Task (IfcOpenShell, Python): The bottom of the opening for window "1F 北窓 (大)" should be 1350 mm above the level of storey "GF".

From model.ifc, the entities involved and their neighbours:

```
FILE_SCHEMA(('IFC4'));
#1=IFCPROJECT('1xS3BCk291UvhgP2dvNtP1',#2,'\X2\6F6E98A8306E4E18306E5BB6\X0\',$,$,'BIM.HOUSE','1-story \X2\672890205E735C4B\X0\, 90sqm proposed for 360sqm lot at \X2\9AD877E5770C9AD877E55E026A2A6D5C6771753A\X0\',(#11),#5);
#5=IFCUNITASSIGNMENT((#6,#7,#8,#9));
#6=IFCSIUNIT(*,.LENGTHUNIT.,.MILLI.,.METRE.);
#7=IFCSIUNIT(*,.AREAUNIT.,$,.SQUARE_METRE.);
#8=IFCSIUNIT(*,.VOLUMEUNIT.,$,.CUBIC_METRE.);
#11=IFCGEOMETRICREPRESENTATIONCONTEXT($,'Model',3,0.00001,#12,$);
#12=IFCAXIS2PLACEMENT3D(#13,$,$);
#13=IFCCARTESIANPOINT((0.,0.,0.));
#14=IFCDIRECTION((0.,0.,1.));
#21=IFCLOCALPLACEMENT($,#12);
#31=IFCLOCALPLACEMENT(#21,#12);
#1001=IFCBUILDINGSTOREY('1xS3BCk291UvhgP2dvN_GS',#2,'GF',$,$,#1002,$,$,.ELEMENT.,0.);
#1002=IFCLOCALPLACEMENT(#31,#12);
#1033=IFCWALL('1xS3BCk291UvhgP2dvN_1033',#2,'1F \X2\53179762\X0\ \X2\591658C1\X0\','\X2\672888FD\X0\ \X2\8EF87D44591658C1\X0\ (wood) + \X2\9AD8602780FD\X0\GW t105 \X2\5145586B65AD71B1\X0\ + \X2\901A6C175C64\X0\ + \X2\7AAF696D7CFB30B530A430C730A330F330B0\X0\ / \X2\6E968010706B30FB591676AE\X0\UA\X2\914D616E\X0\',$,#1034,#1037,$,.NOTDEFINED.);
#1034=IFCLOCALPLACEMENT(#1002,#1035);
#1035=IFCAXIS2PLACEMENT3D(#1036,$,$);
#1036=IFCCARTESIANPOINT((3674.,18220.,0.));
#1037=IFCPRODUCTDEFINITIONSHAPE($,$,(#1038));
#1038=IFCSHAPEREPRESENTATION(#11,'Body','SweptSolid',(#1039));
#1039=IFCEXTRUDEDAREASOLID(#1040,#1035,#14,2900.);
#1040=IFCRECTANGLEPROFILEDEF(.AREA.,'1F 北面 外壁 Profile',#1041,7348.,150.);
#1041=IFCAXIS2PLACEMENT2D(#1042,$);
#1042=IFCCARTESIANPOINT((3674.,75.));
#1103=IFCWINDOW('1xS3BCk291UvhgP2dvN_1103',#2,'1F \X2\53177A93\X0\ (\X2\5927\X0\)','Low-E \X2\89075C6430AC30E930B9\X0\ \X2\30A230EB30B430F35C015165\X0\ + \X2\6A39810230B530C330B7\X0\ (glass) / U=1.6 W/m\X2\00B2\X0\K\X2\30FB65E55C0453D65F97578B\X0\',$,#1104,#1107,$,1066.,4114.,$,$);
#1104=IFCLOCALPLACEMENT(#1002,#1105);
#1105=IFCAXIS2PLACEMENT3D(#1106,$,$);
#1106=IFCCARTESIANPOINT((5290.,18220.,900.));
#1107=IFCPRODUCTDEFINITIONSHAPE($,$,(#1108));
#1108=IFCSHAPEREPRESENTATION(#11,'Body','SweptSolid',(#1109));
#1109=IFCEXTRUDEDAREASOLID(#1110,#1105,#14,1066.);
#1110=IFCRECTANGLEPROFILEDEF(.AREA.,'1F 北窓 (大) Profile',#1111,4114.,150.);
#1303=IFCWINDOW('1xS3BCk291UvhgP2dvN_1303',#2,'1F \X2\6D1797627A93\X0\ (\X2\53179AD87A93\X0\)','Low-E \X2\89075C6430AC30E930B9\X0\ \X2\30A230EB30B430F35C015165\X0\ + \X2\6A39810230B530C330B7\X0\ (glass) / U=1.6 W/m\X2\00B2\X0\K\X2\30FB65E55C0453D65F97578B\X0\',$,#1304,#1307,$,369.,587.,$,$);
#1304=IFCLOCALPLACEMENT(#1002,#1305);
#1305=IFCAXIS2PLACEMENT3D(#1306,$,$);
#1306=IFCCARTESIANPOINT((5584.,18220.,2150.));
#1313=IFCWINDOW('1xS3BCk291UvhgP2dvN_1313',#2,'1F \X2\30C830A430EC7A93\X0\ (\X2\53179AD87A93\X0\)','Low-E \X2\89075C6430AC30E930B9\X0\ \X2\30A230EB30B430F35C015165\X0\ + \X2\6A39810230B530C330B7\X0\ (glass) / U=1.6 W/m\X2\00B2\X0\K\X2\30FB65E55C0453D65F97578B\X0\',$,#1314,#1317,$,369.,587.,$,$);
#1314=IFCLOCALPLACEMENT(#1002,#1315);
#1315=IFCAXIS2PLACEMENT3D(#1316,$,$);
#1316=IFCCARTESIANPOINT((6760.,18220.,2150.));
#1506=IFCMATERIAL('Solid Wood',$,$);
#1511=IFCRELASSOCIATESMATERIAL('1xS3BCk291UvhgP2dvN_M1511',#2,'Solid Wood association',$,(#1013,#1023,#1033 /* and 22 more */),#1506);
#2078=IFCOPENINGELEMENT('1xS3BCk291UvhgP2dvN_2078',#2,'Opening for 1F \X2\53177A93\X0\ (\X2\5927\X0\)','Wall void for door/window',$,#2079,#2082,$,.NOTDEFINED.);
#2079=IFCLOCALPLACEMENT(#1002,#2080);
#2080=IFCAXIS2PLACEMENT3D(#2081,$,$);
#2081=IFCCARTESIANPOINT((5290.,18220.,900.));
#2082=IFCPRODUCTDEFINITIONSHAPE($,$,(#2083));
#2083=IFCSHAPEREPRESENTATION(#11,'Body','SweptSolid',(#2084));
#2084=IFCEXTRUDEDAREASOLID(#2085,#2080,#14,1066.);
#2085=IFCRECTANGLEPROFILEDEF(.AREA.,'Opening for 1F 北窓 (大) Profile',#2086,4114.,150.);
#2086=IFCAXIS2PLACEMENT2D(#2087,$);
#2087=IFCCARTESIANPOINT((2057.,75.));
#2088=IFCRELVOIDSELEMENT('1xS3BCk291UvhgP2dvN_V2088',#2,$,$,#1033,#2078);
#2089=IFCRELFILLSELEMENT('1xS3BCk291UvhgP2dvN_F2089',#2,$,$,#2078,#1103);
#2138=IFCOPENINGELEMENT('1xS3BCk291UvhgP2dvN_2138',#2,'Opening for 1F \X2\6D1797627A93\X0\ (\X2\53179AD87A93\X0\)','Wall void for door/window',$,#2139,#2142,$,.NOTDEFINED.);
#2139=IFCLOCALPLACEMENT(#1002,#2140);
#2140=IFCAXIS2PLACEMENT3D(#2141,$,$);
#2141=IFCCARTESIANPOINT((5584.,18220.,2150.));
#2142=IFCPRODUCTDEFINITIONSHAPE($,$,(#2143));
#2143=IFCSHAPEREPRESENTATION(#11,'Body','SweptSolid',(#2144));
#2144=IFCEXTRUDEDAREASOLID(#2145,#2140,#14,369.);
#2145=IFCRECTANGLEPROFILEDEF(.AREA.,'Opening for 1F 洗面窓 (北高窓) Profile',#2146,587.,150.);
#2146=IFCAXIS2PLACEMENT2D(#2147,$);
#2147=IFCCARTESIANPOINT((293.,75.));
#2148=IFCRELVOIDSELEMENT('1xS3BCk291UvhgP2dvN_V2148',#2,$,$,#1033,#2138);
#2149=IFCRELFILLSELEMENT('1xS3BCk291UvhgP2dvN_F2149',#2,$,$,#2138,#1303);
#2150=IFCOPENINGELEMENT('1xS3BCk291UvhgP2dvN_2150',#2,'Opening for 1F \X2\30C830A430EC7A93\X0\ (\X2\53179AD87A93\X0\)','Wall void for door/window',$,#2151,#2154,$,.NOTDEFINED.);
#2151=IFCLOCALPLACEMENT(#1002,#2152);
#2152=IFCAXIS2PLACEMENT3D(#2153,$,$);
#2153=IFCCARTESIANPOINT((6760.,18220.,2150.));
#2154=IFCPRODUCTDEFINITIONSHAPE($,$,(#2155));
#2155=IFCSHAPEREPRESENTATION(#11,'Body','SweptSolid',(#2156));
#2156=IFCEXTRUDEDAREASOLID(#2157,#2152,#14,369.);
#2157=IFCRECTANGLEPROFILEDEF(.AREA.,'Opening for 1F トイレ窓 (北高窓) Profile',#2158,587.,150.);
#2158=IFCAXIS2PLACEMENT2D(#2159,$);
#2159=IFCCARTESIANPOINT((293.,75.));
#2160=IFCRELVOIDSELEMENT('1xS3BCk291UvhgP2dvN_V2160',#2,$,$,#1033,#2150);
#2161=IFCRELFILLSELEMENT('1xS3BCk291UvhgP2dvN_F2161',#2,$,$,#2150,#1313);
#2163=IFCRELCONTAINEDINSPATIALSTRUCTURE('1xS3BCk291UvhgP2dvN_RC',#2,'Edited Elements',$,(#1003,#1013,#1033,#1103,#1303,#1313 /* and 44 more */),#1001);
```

```python
import numpy as np
import ifcopenshell
import ifcopenshell.api.geometry
import ifcopenshell.geom
import ifcopenshell.util.element
import ifcopenshell.util.placement
import ifcopenshell.util.shape
import ifcopenshell.util.unit

model = ifcopenshell.open("model.ifc")
unit_scale = ifcopenshell.util.unit.calculate_unit_scale(model)

window = model.by_guid("1xS3BCk291UvhgP2dvN_1103")
opening = window.FillsVoids[0].RelatingOpeningElement
storey = ifcopenshell.util.element.get_container(window, ifc_class="IfcBuildingStorey")
level = ifcopenshell.util.placement.get_local_placement(storey.ObjectPlacement)[2, 3]

# The opening's origin need not be at the sill, so measure its lowest point.
shape = ifcopenshell.geom.create_shape(ifcopenshell.geom.settings(), opening)
bottom = ifcopenshell.util.shape.get_shape_bottom_elevation(shape, shape.geometry) / unit_scale
dz = level + 1.35 / unit_scale - bottom

shift = np.array([0.0, 0.0, dz])
# The window is not placed relative to its opening, so move both.
for product in (opening, window):
    matrix = ifcopenshell.util.placement.get_local_placement(product.ObjectPlacement)
    matrix[:3, 3] += shift
    ifcopenshell.api.geometry.edit_object_placement(model, product=product, matrix=matrix, is_si=False)

print(f"moved by {dz * unit_scale:+.3f} m")

model.write("model-out.ifc")
```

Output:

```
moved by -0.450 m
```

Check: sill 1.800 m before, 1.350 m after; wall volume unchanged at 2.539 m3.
